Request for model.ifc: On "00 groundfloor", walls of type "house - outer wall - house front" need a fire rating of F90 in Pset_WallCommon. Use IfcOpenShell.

First a look at what the model holds.

```python
import ifcopenshell
import ifcopenshell.util.element

model = ifcopenshell.open("model.ifc")
print(model.schema)
storey = next(s for s in model.by_type("IfcBuildingStorey") if s.Name == "00 groundfloor")
walls = [e for e in ifcopenshell.util.element.get_decomposition(storey) if e.is_a("IfcWall")]
seen = {}
for e in walls:
    element_type = ifcopenshell.util.element.get_type(e)
    key = (element_type.Name if element_type != e and element_type else None, ifcopenshell.util.element.get_pset(e, "Pset_WallCommon", "FireRating"))
    seen[key] = seen.get(key, 0) + 1
for (name, value), count in sorted(seen.items(), key=str):
    print(count, "x", name, "|", value)
```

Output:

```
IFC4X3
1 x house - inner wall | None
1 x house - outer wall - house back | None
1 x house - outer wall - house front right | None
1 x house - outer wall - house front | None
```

```python
import ifcopenshell
import ifcopenshell.api.pset
import ifcopenshell.util.element

model = ifcopenshell.open("model.ifc")

storey = next(s for s in model.by_type("IfcBuildingStorey") if s.Name == "00 groundfloor")
walls = [e for e in ifcopenshell.util.element.get_decomposition(storey) if e.is_a("IfcWall")]

count = 0
for e in walls:
    element_type = ifcopenshell.util.element.get_type(e)
    if element_type in (None, e) or element_type.Name != "house - outer wall - house front":
        continue
    # add_pset returns the element's existing set when there is one.
    pset = ifcopenshell.api.pset.add_pset(model, product=e, name="Pset_WallCommon")
    ifcopenshell.api.pset.edit_pset(model, pset=pset, properties={"FireRating": "F90"})
    count += 1

print(count, "walls updated")

model.write("model_updated.ifc")
```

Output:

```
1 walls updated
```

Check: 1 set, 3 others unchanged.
